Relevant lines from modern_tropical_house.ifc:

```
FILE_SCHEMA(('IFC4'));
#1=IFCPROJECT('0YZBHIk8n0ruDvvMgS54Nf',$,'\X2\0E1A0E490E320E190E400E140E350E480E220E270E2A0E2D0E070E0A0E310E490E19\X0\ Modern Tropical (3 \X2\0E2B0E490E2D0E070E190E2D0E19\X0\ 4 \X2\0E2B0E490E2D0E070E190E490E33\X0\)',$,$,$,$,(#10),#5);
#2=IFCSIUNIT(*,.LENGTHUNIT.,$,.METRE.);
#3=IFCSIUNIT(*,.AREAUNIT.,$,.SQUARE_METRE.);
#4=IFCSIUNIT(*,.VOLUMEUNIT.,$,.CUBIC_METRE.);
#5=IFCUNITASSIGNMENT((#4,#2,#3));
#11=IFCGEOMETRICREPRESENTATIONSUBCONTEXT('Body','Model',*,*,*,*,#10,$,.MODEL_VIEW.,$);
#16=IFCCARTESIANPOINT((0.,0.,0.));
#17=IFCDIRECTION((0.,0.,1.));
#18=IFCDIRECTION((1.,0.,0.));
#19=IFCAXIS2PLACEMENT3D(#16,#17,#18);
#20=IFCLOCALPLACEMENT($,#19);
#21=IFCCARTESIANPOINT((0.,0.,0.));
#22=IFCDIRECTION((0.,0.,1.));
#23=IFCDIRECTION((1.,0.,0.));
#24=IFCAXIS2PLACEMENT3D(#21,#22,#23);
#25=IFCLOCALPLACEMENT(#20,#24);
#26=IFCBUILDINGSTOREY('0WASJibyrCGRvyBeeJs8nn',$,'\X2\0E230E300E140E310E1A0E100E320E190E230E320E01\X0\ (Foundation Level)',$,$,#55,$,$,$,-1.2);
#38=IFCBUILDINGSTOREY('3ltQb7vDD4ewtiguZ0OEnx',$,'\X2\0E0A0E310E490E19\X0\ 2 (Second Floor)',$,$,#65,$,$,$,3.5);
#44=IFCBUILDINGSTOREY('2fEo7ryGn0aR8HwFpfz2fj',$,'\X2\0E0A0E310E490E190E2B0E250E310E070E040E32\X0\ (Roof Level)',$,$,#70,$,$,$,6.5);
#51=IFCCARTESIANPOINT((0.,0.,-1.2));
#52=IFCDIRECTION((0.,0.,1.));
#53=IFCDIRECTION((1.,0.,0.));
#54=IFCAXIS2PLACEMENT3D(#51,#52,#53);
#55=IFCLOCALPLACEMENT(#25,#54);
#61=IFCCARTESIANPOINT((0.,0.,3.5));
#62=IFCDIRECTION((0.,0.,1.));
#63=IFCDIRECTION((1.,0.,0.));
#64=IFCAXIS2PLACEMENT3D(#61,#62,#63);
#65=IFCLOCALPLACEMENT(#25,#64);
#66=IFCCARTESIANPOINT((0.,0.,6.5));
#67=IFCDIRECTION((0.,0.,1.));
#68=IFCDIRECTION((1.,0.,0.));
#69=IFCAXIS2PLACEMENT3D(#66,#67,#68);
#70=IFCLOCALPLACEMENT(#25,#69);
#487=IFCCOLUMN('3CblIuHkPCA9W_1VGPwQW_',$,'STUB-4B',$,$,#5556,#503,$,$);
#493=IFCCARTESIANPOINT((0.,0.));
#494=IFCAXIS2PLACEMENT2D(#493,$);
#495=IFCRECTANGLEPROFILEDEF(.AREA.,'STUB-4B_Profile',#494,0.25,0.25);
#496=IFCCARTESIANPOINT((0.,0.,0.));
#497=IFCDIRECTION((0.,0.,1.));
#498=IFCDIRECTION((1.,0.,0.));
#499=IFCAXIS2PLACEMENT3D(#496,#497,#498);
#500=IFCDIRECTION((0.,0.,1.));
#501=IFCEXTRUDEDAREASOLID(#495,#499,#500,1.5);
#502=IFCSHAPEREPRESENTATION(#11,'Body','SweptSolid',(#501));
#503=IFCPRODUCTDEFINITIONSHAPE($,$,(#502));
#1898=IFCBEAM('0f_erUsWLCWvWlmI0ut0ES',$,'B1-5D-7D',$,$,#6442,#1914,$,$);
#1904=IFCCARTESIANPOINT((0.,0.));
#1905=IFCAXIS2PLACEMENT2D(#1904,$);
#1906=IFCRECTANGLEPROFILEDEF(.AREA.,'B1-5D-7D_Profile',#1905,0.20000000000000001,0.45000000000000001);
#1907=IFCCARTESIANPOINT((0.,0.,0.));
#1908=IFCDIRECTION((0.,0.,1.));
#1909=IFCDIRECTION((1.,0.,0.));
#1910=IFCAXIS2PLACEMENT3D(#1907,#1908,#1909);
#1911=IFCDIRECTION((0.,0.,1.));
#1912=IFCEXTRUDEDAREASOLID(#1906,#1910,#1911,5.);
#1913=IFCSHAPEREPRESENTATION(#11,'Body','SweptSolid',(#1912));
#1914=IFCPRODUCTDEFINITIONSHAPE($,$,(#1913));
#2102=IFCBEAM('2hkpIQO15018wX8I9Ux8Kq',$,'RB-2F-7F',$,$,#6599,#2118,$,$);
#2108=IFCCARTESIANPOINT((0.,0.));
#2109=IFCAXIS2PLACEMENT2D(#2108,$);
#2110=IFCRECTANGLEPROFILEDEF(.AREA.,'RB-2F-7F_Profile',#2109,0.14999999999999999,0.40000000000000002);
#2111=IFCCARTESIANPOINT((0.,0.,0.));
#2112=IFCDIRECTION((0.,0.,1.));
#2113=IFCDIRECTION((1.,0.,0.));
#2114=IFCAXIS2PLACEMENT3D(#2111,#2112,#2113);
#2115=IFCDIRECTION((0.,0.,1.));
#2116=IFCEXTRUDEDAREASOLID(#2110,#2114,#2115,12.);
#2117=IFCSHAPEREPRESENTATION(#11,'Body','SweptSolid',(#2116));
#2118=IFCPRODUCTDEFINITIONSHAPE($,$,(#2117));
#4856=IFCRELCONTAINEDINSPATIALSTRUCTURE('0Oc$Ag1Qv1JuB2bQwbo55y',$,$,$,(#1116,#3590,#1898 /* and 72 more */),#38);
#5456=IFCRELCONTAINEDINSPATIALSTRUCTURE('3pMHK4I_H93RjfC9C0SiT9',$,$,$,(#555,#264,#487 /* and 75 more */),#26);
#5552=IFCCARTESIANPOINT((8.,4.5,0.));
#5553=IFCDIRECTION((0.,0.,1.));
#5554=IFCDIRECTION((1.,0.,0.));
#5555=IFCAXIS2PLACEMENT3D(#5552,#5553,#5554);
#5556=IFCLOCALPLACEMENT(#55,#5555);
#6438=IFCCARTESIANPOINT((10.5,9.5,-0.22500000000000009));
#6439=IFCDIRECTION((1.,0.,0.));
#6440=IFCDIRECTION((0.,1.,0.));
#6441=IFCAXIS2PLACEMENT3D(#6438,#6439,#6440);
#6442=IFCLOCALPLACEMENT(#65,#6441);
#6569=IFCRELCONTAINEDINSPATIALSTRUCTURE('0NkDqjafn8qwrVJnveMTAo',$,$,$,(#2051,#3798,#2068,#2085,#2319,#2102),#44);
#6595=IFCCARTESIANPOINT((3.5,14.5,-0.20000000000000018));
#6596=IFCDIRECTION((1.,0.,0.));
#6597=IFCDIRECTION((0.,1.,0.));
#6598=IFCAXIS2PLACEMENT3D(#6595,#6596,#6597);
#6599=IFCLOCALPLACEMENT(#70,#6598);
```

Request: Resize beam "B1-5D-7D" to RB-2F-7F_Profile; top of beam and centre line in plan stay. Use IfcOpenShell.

```python
import ifcopenshell
import ifcopenshell.util.element
import ifcopenshell.util.representation

model = ifcopenshell.open("modern_tropical_house.ifc")

member = model.by_id(1898)
source = next(p for p in model.by_type("IfcRectangleProfileDef") if p.ProfileName == "RB-2F-7F_Profile")

body = ifcopenshell.util.representation.get_representation(member, "Model", "Body")
solid = body.Items[0]
old_profile = solid.SweptArea

# Copy the section's sizes but keep this member's own profile position.
profile = ifcopenshell.util.element.copy(model, source)
# Profiles are centred, so shift by half the change in depth to hold the top.
shift = (old_profile.YDim - profile.YDim) / 2
x, y = old_profile.Position.Location.Coordinates
up = (0.0, 1.0)  # upwards, in the solid's own plane
location = model.createIfcCartesianPoint((x + up[0] * shift, y + up[1] * shift))
profile.Position = model.createIfcAxis2Placement2D(location, old_profile.Position.RefDirection)
solid.SweptArea = profile
if not model.get_total_inverses(old_profile):
    ifcopenshell.util.element.remove_deep2(model, old_profile)

print(solid.SweptArea)

model.write("modern_tropical_house_rev.ifc")
```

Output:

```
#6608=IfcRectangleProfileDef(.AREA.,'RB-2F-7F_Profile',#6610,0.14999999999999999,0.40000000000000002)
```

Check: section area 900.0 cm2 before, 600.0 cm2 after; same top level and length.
